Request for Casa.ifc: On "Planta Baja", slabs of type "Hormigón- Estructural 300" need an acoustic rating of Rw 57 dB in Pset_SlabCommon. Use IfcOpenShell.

First a look at what the model holds.

```python
import ifcopenshell
import ifcopenshell.util.element

model = ifcopenshell.open("Casa.ifc")
print(model.schema)
storey = next(s for s in model.by_type("IfcBuildingStorey") if s.Name == "Planta Baja")
slabs = [e for e in ifcopenshell.util.element.get_decomposition(storey) if e.is_a("IfcSlab")]
seen = {}
for e in slabs:
    element_type = ifcopenshell.util.element.get_type(e)
    key = (element_type.Name if element_type != e and element_type else None, ifcopenshell.util.element.get_pset(e, "Pset_SlabCommon", "AcousticRating"))
    seen[key] = seen.get(key, 0) + 1
for (name, value), count in sorted(seen.items(), key=str):
    print(count, "x", name, "|", value)
```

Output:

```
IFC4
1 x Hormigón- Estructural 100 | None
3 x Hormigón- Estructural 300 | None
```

```python
import ifcopenshell
import ifcopenshell.api.pset
import ifcopenshell.util.element

model = ifcopenshell.open("Casa.ifc")

storey = next(s for s in model.by_type("IfcBuildingStorey") if s.Name == "Planta Baja")
slabs = [e for e in ifcopenshell.util.element.get_decomposition(storey) if e.is_a("IfcSlab")]

count = 0
for e in slabs:
    element_type = ifcopenshell.util.element.get_type(e)
    if element_type in (None, e) or element_type.Name != "Hormigón- Estructural 300":
        continue
    # add_pset returns the element's existing set when there is one.
    pset = ifcopenshell.api.pset.add_pset(model, product=e, name="Pset_SlabCommon")
    ifcopenshell.api.pset.edit_pset(model, pset=pset, properties={"AcousticRating": "Rw 57 dB"})
    count += 1

print(count, "slabs updated")

model.write("Casa_v2.ifc")
```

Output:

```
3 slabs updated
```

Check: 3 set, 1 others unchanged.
